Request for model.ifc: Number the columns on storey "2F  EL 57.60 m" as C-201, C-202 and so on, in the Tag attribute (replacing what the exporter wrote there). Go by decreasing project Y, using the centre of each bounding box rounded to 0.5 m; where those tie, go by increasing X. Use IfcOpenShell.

First a look at what the model holds.

```python
import ifcopenshell
import ifcopenshell.util.element
import ifcopenshell.util.placement

model = ifcopenshell.open("model.ifc")
print(model.schema)
storey = next(s for s in model.by_type("IfcBuildingStorey") if s.Name == "2F  EL 57.60 m")
columns = [e for e in ifcopenshell.util.element.get_decomposition(storey) if e.is_a("IfcColumn")]
for e in sorted(columns, key=lambda e: e.id()):
    origin = ifcopenshell.util.placement.get_local_placement(e.ObjectPlacement)[:3, 3]
    print(e.id(), e.Tag, e.Name, origin.round(2) + 0.0, sep=" | ")
```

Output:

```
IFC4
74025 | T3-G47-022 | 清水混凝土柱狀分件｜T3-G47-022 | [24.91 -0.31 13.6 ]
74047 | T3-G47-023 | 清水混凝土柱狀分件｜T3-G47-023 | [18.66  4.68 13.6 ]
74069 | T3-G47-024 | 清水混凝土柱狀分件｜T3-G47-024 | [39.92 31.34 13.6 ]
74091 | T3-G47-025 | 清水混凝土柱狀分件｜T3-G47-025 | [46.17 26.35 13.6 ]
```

```python
import ifcopenshell
import ifcopenshell.geom
import ifcopenshell.util.element
import ifcopenshell.util.shape

model = ifcopenshell.open("model.ifc")
settings = ifcopenshell.geom.settings()
settings.set("use-world-coords", True)


def centre(element):
    shape = ifcopenshell.geom.create_shape(settings, element)
    return ifcopenshell.util.shape.get_bbox_centroid(shape.geometry)


storey = next(s for s in model.by_type("IfcBuildingStorey") if s.Name == "2F  EL 57.60 m")
columns = [e for e in ifcopenshell.util.element.get_decomposition(storey) if e.is_a("IfcColumn")]

# Insertion points can sit at a corner or the storey origin, so sort by the geometry (in metres).
centres = {e: centre(e) for e in columns}
columns.sort(key=lambda e: (-round(centres[e][1] / 0.5), centres[e][0]))

for i, e in enumerate(columns, start=1):
    number = f"C-2{i:02d}"
    e.Tag = number
    print(e.id(), number)

model.write("model_v2.ifc")
```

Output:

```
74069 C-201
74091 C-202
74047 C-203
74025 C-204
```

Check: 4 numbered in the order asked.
